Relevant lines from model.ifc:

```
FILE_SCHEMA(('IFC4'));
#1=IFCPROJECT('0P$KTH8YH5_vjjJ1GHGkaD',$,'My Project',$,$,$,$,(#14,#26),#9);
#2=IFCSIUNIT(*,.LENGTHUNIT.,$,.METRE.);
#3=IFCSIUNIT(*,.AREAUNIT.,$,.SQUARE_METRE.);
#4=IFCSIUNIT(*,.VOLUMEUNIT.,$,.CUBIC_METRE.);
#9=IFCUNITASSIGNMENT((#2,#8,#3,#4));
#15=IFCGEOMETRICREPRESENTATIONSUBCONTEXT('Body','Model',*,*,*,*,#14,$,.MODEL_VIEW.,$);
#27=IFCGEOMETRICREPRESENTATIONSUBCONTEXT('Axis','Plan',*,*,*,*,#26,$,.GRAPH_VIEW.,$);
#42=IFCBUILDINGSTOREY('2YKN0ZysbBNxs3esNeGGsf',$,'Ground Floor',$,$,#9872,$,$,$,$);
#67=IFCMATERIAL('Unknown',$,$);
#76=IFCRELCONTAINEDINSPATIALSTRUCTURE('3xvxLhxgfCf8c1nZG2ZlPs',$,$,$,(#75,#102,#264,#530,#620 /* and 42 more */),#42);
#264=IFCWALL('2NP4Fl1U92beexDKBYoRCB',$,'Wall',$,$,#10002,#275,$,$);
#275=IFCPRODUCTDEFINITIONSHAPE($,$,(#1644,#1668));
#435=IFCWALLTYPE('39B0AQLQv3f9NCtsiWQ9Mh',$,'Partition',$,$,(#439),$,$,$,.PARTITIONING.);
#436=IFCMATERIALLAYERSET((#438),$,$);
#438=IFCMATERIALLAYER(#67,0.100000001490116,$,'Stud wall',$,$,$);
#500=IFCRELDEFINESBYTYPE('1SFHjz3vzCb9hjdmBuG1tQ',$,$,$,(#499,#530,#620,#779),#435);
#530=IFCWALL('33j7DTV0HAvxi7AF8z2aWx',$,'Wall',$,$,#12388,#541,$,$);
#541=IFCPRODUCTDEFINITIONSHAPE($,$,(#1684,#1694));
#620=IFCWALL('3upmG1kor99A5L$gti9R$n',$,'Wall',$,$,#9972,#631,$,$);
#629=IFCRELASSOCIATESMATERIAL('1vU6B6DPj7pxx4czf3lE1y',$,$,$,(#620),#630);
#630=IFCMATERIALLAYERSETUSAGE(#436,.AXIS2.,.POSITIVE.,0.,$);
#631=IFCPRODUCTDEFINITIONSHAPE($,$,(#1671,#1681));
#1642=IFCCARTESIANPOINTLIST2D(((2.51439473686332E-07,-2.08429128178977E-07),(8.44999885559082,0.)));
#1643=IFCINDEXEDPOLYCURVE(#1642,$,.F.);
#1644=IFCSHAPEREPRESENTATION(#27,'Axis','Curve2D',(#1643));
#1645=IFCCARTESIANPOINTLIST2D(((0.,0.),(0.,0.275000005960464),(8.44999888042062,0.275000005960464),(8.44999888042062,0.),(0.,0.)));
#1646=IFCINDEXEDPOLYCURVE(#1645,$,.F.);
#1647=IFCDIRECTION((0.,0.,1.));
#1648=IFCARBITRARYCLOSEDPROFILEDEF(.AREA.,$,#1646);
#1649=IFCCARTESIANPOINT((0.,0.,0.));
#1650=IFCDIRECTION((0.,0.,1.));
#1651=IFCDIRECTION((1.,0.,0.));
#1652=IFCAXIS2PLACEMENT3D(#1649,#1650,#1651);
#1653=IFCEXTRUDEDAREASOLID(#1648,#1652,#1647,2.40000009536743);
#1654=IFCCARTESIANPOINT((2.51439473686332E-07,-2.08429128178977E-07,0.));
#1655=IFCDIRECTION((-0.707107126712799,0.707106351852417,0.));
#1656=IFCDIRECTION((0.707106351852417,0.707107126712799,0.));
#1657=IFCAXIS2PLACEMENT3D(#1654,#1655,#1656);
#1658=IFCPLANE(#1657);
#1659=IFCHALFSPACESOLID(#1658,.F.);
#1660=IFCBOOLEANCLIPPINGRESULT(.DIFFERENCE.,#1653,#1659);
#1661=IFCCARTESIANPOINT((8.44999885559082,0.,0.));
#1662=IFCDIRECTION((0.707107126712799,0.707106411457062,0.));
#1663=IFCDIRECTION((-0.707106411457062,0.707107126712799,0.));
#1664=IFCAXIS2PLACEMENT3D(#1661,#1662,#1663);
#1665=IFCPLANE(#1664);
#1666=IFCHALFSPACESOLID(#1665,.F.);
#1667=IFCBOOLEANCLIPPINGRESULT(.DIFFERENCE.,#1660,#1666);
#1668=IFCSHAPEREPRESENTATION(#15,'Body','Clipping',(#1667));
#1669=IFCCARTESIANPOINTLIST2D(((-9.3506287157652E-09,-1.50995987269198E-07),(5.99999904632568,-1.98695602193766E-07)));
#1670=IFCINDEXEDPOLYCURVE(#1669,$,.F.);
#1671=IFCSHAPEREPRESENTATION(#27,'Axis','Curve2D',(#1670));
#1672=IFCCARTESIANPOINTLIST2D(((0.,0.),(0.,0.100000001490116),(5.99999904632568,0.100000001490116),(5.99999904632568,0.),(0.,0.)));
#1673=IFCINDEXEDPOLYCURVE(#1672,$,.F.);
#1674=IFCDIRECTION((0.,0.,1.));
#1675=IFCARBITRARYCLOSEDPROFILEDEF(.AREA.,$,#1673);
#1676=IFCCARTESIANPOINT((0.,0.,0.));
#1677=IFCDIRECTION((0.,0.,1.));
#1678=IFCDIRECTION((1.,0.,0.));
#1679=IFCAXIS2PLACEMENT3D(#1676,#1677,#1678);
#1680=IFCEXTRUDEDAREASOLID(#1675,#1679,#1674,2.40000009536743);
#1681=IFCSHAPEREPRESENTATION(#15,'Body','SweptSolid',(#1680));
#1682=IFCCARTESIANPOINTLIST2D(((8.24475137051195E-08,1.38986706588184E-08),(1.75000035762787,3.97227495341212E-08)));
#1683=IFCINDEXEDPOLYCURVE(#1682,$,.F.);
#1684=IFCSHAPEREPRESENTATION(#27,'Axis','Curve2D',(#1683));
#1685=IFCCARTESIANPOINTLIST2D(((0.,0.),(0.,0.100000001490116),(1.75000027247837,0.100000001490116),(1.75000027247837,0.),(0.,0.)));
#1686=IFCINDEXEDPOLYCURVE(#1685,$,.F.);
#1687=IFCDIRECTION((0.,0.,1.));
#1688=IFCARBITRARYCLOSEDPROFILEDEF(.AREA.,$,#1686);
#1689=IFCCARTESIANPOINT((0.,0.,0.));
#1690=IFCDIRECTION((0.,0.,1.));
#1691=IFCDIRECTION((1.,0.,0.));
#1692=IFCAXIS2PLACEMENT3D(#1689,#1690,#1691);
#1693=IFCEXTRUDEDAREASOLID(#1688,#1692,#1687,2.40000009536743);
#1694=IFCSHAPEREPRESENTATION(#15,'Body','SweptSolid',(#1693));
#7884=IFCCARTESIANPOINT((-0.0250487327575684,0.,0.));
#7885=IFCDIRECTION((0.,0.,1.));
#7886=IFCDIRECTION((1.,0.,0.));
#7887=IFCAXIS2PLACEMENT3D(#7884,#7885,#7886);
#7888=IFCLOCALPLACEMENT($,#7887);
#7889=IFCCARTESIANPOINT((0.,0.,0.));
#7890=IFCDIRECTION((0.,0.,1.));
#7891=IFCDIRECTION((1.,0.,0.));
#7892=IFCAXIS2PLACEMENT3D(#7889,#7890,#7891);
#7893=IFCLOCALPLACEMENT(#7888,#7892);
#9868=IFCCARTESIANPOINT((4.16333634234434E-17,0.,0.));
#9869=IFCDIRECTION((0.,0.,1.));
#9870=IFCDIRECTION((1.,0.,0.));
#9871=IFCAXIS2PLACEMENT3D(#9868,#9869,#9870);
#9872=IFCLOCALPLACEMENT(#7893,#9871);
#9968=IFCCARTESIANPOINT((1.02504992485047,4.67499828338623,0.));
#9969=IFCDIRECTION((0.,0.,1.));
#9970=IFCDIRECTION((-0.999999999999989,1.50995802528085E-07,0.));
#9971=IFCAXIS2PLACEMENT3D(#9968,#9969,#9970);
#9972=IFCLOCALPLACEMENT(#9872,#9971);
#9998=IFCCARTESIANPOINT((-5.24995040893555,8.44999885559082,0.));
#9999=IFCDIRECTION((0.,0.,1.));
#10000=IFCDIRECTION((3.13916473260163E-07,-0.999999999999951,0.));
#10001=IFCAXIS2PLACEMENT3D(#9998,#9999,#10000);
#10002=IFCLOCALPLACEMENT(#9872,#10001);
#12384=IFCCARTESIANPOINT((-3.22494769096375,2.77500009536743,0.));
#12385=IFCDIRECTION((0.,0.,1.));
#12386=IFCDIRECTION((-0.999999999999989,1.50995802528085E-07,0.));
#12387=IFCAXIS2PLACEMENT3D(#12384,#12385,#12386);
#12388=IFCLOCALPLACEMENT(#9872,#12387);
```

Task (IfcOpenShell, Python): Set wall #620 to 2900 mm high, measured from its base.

```python
import ifcopenshell
import ifcopenshell.geom
import ifcopenshell.util.representation
import ifcopenshell.util.shape
import ifcopenshell.util.unit

model = ifcopenshell.open("model.ifc")
unit_scale = ifcopenshell.util.unit.calculate_unit_scale(model)
settings = ifcopenshell.geom.settings()


def volume(element):
    """Net volume in cubic metres, openings subtracted."""
    shape = ifcopenshell.geom.create_shape(settings, element)
    return ifcopenshell.util.shape.get_volume(shape.geometry)


wall = model.by_guid("3upmG1kor99A5L$gti9R$n")
before = volume(wall)

body = ifcopenshell.util.representation.get_representation(wall, "Model", "Body")
solid = body.Items[0]
old_height = solid.Depth
solid.Depth = 2.9 / unit_scale
after = volume(wall)

print(f"height {old_height:g} -> {solid.Depth:g}, volume {before:.3f} -> {after:.3f} m3")

model.write("model_updated.ifc")
```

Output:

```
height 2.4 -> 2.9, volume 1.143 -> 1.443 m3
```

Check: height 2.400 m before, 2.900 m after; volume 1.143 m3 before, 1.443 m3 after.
